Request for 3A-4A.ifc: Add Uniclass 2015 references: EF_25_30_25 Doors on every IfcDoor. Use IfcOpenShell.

First a look at what the model holds.

```python
import ifcopenshell

model = ifcopenshell.open("3A-4A.ifc")
print(model.schema)
print("classifications:", [c.Name for c in model.by_type("IfcClassification")])
for ifc_class in ("IfcDoor", "IfcRoof", "IfcStair", "IfcWall", "IfcWindow"):
    print(ifc_class, len(model.by_type(ifc_class)))
```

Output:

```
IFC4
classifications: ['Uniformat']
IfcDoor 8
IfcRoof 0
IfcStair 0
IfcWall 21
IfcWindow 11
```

```python
import ifcopenshell
import ifcopenshell.api.classification

model = ifcopenshell.open("3A-4A.ifc")

system = ifcopenshell.api.classification.add_classification(model, classification="Uniclass 2015")

codes = {
    "IfcDoor": ("EF_25_30_25", "Doors"),
}
for ifc_class, (code, name) in codes.items():
    products = model.by_type(ifc_class)
    ifcopenshell.api.classification.add_reference(
        model, products=products, classification=system, identification=code, name=name
    )
    print(code, len(products))

model.write("3A-4A_rev.ifc")
```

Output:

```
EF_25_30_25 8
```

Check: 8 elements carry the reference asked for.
